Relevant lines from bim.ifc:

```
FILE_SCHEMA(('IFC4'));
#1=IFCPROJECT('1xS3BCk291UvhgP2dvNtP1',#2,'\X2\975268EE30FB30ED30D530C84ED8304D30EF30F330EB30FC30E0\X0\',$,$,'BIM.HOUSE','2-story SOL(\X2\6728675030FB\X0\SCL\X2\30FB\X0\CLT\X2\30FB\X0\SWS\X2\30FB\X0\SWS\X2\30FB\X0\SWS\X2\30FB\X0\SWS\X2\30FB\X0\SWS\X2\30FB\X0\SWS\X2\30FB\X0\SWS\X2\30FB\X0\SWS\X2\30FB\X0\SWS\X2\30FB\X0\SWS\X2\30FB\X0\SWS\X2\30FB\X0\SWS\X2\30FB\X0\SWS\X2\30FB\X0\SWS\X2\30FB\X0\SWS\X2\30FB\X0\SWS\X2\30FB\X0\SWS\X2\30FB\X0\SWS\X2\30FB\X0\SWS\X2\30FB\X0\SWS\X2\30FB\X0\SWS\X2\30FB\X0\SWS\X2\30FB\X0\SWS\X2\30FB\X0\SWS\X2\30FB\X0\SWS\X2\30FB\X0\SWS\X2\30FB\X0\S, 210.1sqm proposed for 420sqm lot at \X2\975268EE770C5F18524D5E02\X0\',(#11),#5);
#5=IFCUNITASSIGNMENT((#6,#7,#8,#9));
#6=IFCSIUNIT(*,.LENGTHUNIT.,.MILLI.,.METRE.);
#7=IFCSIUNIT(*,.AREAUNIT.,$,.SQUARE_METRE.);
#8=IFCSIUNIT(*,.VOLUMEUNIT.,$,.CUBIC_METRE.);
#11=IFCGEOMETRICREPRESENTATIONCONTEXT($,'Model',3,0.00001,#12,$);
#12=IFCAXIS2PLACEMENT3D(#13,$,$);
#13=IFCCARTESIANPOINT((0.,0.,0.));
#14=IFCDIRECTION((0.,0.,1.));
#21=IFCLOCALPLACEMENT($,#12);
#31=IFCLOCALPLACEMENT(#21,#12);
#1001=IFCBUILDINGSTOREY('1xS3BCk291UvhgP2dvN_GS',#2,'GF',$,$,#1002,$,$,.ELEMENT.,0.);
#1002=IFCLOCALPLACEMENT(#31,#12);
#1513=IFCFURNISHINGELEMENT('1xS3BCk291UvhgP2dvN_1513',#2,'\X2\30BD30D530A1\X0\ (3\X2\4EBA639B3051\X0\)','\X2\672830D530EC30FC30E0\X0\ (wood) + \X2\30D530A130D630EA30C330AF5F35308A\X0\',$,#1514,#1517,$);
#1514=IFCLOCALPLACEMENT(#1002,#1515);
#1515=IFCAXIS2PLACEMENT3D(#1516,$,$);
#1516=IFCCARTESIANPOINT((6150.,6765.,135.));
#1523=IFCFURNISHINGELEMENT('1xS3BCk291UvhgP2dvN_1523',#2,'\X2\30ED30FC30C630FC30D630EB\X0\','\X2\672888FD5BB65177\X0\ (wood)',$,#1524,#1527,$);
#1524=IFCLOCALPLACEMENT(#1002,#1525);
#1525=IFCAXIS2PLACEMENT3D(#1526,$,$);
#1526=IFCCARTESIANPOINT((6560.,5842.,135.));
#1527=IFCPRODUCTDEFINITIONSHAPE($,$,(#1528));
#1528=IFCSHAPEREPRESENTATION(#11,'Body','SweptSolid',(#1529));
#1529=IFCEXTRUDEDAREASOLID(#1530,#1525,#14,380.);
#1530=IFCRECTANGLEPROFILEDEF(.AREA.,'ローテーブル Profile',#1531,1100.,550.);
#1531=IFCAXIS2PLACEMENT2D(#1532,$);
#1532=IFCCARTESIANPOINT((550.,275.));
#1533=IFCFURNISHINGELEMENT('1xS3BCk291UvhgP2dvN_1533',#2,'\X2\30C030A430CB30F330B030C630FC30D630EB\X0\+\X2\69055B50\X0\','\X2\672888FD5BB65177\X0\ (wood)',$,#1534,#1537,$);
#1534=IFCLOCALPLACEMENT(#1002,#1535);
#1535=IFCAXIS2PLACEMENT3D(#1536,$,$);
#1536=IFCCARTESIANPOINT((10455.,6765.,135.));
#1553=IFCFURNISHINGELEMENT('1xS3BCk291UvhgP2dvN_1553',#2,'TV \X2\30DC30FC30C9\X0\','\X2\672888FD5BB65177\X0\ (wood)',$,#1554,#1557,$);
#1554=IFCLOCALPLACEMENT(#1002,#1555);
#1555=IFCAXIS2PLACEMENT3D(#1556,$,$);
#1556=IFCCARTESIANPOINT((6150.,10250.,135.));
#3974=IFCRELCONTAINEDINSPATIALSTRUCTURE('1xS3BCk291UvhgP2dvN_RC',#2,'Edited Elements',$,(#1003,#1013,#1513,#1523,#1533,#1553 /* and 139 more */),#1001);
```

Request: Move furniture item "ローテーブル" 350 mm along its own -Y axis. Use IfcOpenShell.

```python
import ifcopenshell
import ifcopenshell.api.geometry
import ifcopenshell.util.placement

model = ifcopenshell.open("bim.ifc")

item = model.by_guid("1xS3BCk291UvhgP2dvN_1523")
matrix = ifcopenshell.util.placement.get_local_placement(item.ObjectPlacement)
matrix[:3, 3] -= matrix[:3, 1] * 350.0
ifcopenshell.api.geometry.edit_object_placement(model, product=item, matrix=matrix, is_si=False)

print(ifcopenshell.util.placement.get_local_placement(item.ObjectPlacement).round(3) + 0.0)

model.write("bim_updated.ifc")
```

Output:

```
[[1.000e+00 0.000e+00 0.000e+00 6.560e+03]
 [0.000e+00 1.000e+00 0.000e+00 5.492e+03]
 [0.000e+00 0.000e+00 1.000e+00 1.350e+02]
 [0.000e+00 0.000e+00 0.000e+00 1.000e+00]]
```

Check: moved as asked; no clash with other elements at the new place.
